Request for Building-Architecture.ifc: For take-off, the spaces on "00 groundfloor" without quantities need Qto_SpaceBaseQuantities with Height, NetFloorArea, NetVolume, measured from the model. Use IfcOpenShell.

First a look at what the model holds.

```python
import ifcopenshell
import ifcopenshell.util.element
import ifcopenshell.util.unit

model = ifcopenshell.open("Building-Architecture.ifc")
print(model.schema)
for unit_type in ("LENGTHUNIT", "AREAUNIT", "VOLUMEUNIT"):
    print(unit_type, ifcopenshell.util.unit.calculate_unit_scale(model, unit_type))
storey = next(s for s in model.by_type("IfcBuildingStorey") if s.Name == "00 groundfloor")
spaces = [e for e in ifcopenshell.util.element.get_decomposition(storey) if e.is_a("IfcSpace")]
for e in sorted(spaces, key=lambda e: e.id()):
    print(e.id(), e.is_a(), e.Name, list(ifcopenshell.util.element.get_psets(e, qtos_only=True)), sep=" | ")
```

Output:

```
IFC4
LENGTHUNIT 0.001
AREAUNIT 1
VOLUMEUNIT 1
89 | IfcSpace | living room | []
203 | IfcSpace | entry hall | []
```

```python
import ifcopenshell
import ifcopenshell.api.pset
import ifcopenshell.geom
import ifcopenshell.util.element
import ifcopenshell.util.shape
import ifcopenshell.util.unit

model = ifcopenshell.open("Building-Architecture.ifc")
unit_scale = ifcopenshell.util.unit.calculate_unit_scale(model)
area_scale = ifcopenshell.util.unit.calculate_unit_scale(model, "AREAUNIT")
volume_scale = ifcopenshell.util.unit.calculate_unit_scale(model, "VOLUMEUNIT")
settings = ifcopenshell.geom.settings()

storey = next(s for s in model.by_type("IfcBuildingStorey") if s.Name == "00 groundfloor")
spaces = [e for e in ifcopenshell.util.element.get_decomposition(storey) if e.is_a("IfcSpace")]

for e in sorted(spaces, key=lambda e: e.id()):
    if ifcopenshell.util.element.get_psets(e, qtos_only=True, should_inherit=False):
        continue
    # Geometry comes back in metres, in the element's own axes.
    shape = ifcopenshell.geom.create_shape(settings, e)
    values = {
        "Height": ifcopenshell.util.shape.get_z(shape.geometry) / unit_scale,
        "NetFloorArea": ifcopenshell.util.shape.get_footprint_area(shape.geometry) / area_scale,
        "NetVolume": ifcopenshell.util.shape.get_volume(shape.geometry) / volume_scale,
    }
    qto = ifcopenshell.api.pset.add_qto(model, product=e, name="Qto_SpaceBaseQuantities")
    ifcopenshell.api.pset.edit_qto(model, qto=qto, properties=values)
    print(e.id(), {k: round(v, 3) for k, v in values.items()})

model.write("Building-Architecture-out.ifc")
```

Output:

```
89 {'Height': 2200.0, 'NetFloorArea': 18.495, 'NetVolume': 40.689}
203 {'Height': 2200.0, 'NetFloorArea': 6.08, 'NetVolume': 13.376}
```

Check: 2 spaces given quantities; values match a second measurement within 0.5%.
